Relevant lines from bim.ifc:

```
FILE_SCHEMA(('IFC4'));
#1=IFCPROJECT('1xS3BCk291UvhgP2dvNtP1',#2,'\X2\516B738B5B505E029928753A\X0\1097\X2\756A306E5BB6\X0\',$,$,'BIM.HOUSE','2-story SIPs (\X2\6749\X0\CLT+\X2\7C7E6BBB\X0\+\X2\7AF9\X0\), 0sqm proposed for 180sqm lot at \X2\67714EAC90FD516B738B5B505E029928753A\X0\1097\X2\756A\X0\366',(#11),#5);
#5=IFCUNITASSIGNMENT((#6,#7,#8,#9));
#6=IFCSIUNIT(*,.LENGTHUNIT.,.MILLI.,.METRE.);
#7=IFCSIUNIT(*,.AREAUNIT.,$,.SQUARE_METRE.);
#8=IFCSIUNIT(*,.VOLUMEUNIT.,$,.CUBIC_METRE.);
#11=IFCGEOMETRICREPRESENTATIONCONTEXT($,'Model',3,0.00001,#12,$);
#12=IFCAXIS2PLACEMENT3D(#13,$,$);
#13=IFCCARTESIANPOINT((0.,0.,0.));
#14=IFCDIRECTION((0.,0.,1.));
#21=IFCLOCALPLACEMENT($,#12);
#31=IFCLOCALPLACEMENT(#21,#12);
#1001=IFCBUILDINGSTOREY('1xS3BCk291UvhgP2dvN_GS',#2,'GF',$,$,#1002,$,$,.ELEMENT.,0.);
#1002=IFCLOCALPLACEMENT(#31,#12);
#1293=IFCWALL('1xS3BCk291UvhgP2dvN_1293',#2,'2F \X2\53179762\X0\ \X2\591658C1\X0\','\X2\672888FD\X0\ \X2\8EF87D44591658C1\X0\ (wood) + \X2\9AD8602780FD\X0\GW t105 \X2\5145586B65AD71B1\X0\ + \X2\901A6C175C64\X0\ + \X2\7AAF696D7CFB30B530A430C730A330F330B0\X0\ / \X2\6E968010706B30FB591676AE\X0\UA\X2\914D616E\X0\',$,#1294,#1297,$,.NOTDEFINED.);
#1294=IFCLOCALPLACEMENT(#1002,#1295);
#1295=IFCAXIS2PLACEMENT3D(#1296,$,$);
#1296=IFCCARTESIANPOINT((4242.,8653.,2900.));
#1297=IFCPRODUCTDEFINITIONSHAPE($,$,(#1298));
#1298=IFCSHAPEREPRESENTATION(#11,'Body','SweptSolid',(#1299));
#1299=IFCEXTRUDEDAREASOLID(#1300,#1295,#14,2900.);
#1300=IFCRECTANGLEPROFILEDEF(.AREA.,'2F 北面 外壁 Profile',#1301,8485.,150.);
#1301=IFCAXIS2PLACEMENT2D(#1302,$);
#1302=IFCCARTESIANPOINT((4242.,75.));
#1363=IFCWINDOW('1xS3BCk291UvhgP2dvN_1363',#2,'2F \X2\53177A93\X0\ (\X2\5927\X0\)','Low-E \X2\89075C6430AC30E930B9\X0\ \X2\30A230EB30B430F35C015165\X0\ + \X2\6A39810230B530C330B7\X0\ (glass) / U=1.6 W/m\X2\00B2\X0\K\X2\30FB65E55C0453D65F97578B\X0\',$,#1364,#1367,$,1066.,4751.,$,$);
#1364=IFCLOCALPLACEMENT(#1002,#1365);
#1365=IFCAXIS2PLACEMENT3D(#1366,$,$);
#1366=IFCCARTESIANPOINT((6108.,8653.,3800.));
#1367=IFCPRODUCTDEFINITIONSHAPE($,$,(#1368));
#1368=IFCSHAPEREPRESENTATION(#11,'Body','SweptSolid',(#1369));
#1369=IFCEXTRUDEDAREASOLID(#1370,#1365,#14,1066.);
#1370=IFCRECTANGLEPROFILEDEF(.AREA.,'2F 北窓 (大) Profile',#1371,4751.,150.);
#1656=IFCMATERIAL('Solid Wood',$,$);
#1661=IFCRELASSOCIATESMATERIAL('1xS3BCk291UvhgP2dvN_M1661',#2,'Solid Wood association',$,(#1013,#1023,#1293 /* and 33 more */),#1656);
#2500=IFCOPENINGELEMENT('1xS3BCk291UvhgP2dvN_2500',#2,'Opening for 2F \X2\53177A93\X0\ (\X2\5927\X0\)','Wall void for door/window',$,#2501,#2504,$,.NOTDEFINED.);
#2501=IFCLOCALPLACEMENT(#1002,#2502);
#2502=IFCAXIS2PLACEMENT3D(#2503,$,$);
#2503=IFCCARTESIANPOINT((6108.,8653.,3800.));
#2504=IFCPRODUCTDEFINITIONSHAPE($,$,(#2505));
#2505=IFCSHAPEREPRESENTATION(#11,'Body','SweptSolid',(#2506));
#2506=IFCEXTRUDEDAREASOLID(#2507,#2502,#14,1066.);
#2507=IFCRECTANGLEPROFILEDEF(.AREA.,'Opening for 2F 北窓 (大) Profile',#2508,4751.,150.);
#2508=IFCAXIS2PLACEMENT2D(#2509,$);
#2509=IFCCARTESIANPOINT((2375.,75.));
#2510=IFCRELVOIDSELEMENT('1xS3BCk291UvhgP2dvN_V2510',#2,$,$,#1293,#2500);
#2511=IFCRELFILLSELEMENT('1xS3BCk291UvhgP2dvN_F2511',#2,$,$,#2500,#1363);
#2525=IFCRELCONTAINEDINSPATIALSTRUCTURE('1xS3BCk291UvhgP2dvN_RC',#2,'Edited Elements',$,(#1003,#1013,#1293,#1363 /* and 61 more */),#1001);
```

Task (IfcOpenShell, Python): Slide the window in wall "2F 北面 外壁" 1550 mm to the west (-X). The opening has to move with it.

```python
import ifcopenshell
import ifcopenshell.api.geometry
import ifcopenshell.util.placement

model = ifcopenshell.open("bim.ifc")

window = model.by_id(1363)
opening = window.FillsVoids[0].RelatingOpeningElement
wall = opening.VoidsElements[0].RelatingBuildingElement

wall_matrix = ifcopenshell.util.placement.get_local_placement(wall.ObjectPlacement)
shift = wall_matrix[:3, 0] * -1550.0
before = ifcopenshell.util.placement.get_local_placement(window.ObjectPlacement)[:3, 3].copy()

# The window is not placed relative to its opening, so move both.
for product in (opening, window):
    matrix = ifcopenshell.util.placement.get_local_placement(product.ObjectPlacement)
    matrix[:3, 3] += shift
    ifcopenshell.api.geometry.edit_object_placement(model, product=product, matrix=matrix, is_si=False)

after = ifcopenshell.util.placement.get_local_placement(window.ObjectPlacement)[:3, 3]
print("window moved by", (after - before).round(3) + 0.0)

model.write("bim_edited.ifc")
```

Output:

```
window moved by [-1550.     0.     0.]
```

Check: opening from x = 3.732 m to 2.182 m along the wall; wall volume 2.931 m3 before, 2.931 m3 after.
